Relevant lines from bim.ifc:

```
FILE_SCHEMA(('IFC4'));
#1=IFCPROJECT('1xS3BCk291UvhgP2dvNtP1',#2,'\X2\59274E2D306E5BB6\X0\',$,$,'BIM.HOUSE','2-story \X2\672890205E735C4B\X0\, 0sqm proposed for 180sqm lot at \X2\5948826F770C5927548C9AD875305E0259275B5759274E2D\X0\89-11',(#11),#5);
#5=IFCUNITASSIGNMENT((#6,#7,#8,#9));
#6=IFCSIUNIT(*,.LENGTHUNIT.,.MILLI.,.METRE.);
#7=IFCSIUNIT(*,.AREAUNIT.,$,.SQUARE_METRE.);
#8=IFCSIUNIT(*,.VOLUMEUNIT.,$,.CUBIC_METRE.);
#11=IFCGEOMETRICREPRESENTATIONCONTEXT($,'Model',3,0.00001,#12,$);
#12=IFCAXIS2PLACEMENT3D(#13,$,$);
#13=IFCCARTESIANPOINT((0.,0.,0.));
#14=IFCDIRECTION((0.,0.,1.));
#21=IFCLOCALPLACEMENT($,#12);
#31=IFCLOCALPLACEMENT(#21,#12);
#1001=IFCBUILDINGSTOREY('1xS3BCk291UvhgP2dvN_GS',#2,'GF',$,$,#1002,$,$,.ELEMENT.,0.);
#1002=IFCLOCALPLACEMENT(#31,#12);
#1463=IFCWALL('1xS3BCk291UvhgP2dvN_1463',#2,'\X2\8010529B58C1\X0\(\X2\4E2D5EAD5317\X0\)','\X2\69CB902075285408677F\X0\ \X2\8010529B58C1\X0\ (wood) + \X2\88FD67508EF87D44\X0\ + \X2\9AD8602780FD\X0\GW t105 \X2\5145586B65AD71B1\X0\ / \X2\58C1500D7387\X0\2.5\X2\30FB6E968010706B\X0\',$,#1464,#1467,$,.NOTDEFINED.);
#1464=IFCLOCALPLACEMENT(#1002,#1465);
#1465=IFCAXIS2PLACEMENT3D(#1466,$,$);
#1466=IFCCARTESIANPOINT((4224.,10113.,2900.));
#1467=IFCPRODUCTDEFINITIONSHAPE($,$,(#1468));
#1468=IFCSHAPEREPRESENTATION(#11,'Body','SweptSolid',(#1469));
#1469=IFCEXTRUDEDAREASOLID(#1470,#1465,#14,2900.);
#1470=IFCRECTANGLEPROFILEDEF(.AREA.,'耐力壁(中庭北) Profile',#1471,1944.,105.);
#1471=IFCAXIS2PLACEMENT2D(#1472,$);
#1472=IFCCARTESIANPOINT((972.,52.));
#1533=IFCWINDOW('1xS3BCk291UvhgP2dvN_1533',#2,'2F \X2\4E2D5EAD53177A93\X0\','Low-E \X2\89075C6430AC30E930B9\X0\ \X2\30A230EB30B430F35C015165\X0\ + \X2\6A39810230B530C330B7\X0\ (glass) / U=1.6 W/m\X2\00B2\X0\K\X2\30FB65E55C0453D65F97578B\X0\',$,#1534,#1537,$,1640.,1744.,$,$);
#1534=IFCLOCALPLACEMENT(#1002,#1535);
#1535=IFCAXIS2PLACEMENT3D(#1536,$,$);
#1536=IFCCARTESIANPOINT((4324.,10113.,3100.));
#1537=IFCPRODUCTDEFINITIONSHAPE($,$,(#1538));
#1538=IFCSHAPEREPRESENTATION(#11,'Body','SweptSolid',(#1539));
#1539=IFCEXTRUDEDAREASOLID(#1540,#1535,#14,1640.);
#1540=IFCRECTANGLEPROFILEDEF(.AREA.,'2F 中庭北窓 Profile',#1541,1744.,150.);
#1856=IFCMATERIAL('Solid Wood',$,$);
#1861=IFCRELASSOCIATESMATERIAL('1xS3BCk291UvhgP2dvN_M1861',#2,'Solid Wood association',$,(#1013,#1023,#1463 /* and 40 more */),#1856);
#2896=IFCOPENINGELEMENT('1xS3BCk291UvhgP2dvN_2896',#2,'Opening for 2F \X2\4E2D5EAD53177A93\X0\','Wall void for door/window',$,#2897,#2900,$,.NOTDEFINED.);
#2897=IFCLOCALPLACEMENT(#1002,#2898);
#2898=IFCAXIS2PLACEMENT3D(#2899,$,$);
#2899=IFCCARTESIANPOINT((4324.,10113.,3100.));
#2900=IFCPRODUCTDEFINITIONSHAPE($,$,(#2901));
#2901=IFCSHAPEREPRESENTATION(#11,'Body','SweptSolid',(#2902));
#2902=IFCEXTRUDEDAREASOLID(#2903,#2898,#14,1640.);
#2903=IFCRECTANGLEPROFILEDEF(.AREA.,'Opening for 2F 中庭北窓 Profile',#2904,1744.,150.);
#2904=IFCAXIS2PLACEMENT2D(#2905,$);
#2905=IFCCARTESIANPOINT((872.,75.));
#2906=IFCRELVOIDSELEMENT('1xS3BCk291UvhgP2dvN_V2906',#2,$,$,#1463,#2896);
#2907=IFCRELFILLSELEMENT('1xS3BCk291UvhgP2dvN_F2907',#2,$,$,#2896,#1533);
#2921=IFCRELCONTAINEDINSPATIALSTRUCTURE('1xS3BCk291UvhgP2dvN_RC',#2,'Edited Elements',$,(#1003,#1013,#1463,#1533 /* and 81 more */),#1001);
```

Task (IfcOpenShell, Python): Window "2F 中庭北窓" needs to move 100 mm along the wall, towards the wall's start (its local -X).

```python
import ifcopenshell
import ifcopenshell.api.geometry
import ifcopenshell.util.placement

model = ifcopenshell.open("bim.ifc")

window = model.by_id(1533)
opening = window.FillsVoids[0].RelatingOpeningElement
wall = opening.VoidsElements[0].RelatingBuildingElement

wall_matrix = ifcopenshell.util.placement.get_local_placement(wall.ObjectPlacement)
shift = wall_matrix[:3, 0] * -100.0
before = ifcopenshell.util.placement.get_local_placement(window.ObjectPlacement)[:3, 3].copy()

# The window is not placed relative to its opening, so move both.
for product in (opening, window):
    matrix = ifcopenshell.util.placement.get_local_placement(product.ObjectPlacement)
    matrix[:3, 3] += shift
    ifcopenshell.api.geometry.edit_object_placement(model, product=product, matrix=matrix, is_si=False)

after = ifcopenshell.util.placement.get_local_placement(window.ObjectPlacement)[:3, 3]
print("window moved by", (after - before).round(3) + 0.0)

model.write("bim_v2.ifc")
```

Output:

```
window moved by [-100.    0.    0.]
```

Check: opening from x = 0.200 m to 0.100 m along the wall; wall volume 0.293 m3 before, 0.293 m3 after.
